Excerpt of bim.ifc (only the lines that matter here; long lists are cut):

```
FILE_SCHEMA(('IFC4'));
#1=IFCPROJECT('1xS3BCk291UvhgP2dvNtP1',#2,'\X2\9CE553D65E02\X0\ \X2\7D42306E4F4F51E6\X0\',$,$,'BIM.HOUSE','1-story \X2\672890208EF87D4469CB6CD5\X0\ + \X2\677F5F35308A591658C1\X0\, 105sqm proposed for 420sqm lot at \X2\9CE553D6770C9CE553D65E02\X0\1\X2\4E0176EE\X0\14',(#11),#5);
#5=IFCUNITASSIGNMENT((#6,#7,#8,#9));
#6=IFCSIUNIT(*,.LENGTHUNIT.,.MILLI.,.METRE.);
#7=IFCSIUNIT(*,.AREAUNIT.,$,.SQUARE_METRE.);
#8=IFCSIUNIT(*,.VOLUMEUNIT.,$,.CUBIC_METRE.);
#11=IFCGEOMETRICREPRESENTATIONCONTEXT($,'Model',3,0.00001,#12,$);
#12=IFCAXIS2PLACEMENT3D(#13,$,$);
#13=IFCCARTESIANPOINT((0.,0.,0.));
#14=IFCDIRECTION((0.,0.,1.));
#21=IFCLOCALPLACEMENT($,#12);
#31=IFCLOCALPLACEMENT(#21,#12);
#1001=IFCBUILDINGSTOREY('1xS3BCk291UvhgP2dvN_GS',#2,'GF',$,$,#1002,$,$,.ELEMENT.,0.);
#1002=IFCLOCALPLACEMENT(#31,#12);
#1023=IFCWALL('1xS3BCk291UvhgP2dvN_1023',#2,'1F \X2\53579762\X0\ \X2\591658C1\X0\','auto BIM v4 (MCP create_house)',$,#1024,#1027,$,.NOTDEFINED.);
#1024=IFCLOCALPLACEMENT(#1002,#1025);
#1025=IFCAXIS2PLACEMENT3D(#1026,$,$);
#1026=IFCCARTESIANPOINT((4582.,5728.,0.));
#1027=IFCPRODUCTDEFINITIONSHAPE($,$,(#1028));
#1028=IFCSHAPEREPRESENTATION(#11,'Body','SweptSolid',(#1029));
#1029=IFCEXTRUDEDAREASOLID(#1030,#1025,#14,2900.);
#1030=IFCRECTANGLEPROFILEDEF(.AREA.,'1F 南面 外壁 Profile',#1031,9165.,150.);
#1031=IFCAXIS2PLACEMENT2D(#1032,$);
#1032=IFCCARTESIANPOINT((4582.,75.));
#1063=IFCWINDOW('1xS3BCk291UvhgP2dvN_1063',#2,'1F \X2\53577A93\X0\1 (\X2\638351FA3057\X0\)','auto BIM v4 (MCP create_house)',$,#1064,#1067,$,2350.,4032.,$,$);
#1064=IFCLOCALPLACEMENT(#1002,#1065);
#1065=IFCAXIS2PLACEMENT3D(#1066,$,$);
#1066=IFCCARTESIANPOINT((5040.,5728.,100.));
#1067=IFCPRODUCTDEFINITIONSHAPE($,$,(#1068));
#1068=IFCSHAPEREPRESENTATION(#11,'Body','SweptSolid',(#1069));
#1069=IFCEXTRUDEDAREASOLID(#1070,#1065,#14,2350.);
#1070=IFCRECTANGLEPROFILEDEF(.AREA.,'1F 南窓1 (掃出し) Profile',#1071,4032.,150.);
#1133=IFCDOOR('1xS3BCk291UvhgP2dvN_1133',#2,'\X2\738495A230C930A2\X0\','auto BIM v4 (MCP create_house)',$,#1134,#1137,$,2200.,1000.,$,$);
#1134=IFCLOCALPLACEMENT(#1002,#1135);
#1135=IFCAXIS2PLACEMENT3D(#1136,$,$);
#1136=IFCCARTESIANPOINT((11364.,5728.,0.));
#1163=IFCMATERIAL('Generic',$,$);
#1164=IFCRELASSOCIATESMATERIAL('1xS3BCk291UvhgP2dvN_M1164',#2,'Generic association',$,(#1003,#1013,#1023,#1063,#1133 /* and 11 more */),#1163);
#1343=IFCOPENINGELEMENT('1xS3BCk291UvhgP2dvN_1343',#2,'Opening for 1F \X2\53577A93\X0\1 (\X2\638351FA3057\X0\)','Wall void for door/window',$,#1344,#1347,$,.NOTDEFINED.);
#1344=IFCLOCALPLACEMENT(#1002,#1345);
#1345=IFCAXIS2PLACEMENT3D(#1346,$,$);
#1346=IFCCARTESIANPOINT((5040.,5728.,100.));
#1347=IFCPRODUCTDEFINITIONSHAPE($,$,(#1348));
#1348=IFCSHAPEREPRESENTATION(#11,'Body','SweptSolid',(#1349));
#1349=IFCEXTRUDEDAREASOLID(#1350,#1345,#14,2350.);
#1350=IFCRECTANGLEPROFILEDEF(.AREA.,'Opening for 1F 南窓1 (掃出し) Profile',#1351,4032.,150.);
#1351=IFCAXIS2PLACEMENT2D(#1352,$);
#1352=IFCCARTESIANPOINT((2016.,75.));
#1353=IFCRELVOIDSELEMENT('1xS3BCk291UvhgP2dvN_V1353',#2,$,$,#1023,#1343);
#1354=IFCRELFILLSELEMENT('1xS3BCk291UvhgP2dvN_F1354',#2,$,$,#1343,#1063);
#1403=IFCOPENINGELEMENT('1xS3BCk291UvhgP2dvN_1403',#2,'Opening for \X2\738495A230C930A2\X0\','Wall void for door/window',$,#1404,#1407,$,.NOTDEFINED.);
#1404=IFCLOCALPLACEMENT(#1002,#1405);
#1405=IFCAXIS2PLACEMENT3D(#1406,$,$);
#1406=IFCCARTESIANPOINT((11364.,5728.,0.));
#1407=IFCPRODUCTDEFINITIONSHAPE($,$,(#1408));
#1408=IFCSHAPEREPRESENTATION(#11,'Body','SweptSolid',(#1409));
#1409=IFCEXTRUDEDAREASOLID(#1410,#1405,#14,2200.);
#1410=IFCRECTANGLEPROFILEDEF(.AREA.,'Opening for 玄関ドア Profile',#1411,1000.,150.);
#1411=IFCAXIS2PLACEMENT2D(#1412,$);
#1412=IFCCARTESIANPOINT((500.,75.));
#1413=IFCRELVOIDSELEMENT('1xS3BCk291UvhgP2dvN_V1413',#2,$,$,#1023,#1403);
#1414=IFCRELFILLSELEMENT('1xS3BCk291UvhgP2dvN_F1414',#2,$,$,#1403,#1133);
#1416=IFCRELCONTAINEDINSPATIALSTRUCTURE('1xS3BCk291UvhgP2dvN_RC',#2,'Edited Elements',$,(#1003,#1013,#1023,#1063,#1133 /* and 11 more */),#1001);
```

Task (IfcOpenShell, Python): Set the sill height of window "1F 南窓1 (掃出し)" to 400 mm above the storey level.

```python
import numpy as np
import ifcopenshell
import ifcopenshell.api.geometry
import ifcopenshell.geom
import ifcopenshell.util.element
import ifcopenshell.util.placement
import ifcopenshell.util.shape
import ifcopenshell.util.unit

model = ifcopenshell.open("bim.ifc")
unit_scale = ifcopenshell.util.unit.calculate_unit_scale(model)

window = model.by_guid("1xS3BCk291UvhgP2dvN_1063")
opening = window.FillsVoids[0].RelatingOpeningElement
storey = ifcopenshell.util.element.get_container(window, ifc_class="IfcBuildingStorey")
level = ifcopenshell.util.placement.get_local_placement(storey.ObjectPlacement)[2, 3]

# The opening's origin need not be at the sill, so measure its lowest point.
shape = ifcopenshell.geom.create_shape(ifcopenshell.geom.settings(), opening)
bottom = ifcopenshell.util.shape.get_shape_bottom_elevation(shape, shape.geometry) / unit_scale
dz = level + 0.4 / unit_scale - bottom

shift = np.array([0.0, 0.0, dz])
# The window is not placed relative to its opening, so move both.
for product in (opening, window):
    matrix = ifcopenshell.util.placement.get_local_placement(product.ObjectPlacement)
    matrix[:3, 3] += shift
    ifcopenshell.api.geometry.edit_object_placement(model, product=product, matrix=matrix, is_si=False)

print(f"moved by {dz * unit_scale:+.3f} m")

model.write("bim_v2.ifc")
```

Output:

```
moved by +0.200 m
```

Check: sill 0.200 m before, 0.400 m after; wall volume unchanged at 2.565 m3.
